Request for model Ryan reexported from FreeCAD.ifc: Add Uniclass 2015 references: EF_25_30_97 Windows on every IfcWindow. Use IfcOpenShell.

First a look at what the model holds.

```python
import ifcopenshell

model = ifcopenshell.open("model Ryan reexported from FreeCAD.ifc")
print(model.schema)
print("classifications:", [c.Name for c in model.by_type("IfcClassification")])
for ifc_class in ("IfcDoor", "IfcRoof", "IfcStair", "IfcWall", "IfcWindow"):
    print(ifc_class, len(model.by_type(ifc_class)))
```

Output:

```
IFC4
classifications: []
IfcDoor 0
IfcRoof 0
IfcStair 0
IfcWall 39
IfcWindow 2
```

```python
import ifcopenshell
import ifcopenshell.api.classification

model = ifcopenshell.open("model Ryan reexported from FreeCAD.ifc")

system = ifcopenshell.api.classification.add_classification(model, classification="Uniclass 2015")

codes = {
    "IfcWindow": ("EF_25_30_97", "Windows"),
}
for ifc_class, (code, name) in codes.items():
    products = model.by_type(ifc_class)
    ifcopenshell.api.classification.add_reference(
        model, products=products, classification=system, identification=code, name=name
    )
    print(code, len(products))

model.write("model Ryan reexported from FreeCAD_v2.ifc")
```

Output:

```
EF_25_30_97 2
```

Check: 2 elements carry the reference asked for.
